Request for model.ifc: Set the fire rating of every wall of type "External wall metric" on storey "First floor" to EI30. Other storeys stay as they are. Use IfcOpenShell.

First a look at what the model holds.

```python
import ifcopenshell
import ifcopenshell.util.element

model = ifcopenshell.open("model.ifc")
print(model.schema)
storey = next(s for s in model.by_type("IfcBuildingStorey") if s.Name == "First floor")
walls = [e for e in ifcopenshell.util.element.get_decomposition(storey) if e.is_a("IfcWall")]
seen = {}
for e in walls:
    element_type = ifcopenshell.util.element.get_type(e)
    key = (element_type.Name if element_type != e and element_type else None, ifcopenshell.util.element.get_pset(e, "Pset_WallCommon", "FireRating"))
    seen[key] = seen.get(key, 0) + 1
for (name, value), count in sorted(seen.items(), key=str):
    print(count, "x", name, "|", value)
```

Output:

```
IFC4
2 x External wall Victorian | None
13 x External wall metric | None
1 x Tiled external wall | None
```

```python
import ifcopenshell
import ifcopenshell.api.pset
import ifcopenshell.util.element

model = ifcopenshell.open("model.ifc")

storey = next(s for s in model.by_type("IfcBuildingStorey") if s.Name == "First floor")
walls = [e for e in ifcopenshell.util.element.get_decomposition(storey) if e.is_a("IfcWall")]

count = 0
for e in walls:
    element_type = ifcopenshell.util.element.get_type(e)
    if element_type in (None, e) or element_type.Name != "External wall metric":
        continue
    # add_pset returns the element's existing set when there is one.
    pset = ifcopenshell.api.pset.add_pset(model, product=e, name="Pset_WallCommon")
    ifcopenshell.api.pset.edit_pset(model, pset=pset, properties={"FireRating": "EI30"})
    count += 1

print(count, "walls updated")

model.write("model_edited.ifc")
```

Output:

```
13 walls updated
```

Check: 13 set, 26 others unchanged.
